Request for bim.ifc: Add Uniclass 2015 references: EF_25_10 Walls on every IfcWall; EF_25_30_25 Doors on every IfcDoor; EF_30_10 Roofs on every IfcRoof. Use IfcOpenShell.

First a look at what the model holds.

```python
import ifcopenshell

model = ifcopenshell.open("bim.ifc")
print(model.schema)
print("classifications:", [c.Name for c in model.by_type("IfcClassification")])
for ifc_class in ("IfcDoor", "IfcRoof", "IfcStair", "IfcWall", "IfcWindow"):
    print(ifc_class, len(model.by_type(ifc_class)))
```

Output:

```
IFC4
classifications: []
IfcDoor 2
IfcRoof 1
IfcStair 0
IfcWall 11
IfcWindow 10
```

```python
import ifcopenshell
import ifcopenshell.api.classification

model = ifcopenshell.open("bim.ifc")

system = ifcopenshell.api.classification.add_classification(model, classification="Uniclass 2015")

codes = {
    "IfcWall": ("EF_25_10", "Walls"),
    "IfcDoor": ("EF_25_30_25", "Doors"),
    "IfcRoof": ("EF_30_10", "Roofs"),
}
for ifc_class, (code, name) in codes.items():
    products = model.by_type(ifc_class)
    ifcopenshell.api.classification.add_reference(
        model, products=products, classification=system, identification=code, name=name
    )
    print(code, len(products))

model.write("bim_updated.ifc")
```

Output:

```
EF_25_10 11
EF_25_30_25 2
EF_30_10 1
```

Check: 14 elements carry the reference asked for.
